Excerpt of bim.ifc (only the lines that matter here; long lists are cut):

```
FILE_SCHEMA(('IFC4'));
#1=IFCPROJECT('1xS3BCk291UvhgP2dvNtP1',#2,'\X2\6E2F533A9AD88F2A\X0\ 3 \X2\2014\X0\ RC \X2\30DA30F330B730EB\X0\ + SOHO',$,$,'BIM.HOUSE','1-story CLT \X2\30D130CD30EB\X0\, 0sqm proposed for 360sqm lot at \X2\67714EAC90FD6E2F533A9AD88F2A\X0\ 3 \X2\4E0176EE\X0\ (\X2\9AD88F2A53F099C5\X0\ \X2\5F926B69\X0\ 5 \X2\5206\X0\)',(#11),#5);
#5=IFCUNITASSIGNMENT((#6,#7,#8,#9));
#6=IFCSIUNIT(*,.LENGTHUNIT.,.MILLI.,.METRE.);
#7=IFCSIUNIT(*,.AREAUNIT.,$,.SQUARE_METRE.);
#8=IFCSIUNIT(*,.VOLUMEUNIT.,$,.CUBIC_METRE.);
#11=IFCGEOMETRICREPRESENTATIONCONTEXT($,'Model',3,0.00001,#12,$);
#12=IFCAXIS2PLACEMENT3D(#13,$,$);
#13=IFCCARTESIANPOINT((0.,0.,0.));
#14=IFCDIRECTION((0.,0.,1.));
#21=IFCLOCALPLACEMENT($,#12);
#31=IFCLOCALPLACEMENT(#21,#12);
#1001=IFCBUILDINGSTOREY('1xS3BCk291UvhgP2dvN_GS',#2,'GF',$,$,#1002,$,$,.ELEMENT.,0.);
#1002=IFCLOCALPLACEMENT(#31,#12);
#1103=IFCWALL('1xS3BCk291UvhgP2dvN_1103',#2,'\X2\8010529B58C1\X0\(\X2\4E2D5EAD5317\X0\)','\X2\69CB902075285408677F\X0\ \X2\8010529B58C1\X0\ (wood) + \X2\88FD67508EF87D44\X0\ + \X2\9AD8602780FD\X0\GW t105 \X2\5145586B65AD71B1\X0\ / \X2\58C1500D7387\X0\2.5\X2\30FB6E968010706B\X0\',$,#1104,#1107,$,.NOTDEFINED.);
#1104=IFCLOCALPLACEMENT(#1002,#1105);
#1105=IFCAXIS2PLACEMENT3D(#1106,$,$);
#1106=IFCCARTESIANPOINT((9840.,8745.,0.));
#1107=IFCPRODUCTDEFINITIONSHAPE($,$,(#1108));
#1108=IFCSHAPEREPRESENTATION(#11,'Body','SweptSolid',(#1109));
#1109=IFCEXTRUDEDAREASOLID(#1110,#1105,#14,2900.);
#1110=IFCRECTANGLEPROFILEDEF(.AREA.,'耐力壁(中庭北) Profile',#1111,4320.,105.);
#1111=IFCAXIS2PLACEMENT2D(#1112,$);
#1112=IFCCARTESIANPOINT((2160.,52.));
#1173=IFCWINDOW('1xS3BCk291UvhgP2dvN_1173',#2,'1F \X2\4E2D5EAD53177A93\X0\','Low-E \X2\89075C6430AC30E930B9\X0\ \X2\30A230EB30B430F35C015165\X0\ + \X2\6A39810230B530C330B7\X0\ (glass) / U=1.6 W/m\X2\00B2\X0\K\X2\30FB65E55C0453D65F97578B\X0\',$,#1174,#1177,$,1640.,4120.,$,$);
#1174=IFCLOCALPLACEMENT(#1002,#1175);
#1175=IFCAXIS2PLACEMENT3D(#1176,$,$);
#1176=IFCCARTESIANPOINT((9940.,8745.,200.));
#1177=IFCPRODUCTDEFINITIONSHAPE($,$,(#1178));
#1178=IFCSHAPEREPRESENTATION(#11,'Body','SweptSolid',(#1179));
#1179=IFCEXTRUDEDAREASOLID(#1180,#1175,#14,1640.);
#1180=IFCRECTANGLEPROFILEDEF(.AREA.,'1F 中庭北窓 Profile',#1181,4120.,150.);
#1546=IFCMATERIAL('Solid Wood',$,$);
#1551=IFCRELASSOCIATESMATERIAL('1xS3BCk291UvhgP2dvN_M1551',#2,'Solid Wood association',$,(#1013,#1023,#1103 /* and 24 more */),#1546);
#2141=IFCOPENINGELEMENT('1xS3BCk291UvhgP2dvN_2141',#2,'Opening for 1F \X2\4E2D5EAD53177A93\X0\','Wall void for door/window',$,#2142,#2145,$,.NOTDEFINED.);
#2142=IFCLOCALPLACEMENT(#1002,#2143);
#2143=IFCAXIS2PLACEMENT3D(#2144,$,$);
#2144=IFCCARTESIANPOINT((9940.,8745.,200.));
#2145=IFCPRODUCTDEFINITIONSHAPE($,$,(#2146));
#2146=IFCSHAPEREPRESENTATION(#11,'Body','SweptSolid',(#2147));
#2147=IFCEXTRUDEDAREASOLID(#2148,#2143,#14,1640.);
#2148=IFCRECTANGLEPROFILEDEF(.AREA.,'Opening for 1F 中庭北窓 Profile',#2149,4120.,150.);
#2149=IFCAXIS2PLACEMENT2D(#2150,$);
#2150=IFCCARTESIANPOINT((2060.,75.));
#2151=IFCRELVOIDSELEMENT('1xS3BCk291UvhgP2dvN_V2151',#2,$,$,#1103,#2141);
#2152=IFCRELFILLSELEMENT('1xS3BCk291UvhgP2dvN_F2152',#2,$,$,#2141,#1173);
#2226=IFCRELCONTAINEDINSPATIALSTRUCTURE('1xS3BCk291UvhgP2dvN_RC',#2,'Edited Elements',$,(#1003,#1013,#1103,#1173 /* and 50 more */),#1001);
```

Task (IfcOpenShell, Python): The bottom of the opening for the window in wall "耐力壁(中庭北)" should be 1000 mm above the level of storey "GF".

```python
import numpy as np
import ifcopenshell
import ifcopenshell.api.geometry
import ifcopenshell.geom
import ifcopenshell.util.element
import ifcopenshell.util.placement
import ifcopenshell.util.shape
import ifcopenshell.util.unit

model = ifcopenshell.open("bim.ifc")
unit_scale = ifcopenshell.util.unit.calculate_unit_scale(model)

window = model.by_id(1173)
opening = window.FillsVoids[0].RelatingOpeningElement
storey = ifcopenshell.util.element.get_container(window, ifc_class="IfcBuildingStorey")
level = ifcopenshell.util.placement.get_local_placement(storey.ObjectPlacement)[2, 3]

# The opening's origin need not be at the sill, so measure its lowest point.
shape = ifcopenshell.geom.create_shape(ifcopenshell.geom.settings(), opening)
bottom = ifcopenshell.util.shape.get_shape_bottom_elevation(shape, shape.geometry) / unit_scale
dz = level + 1000.0 - bottom

shift = np.array([0.0, 0.0, dz])
# The window is not placed relative to its opening, so move both.
for product in (opening, window):
    matrix = ifcopenshell.util.placement.get_local_placement(product.ObjectPlacement)
    matrix[:3, 3] += shift
    ifcopenshell.api.geometry.edit_object_placement(model, product=product, matrix=matrix, is_si=False)

print(f"moved by {dz * unit_scale:+.3f} m")

model.write("bim_v2.ifc")
```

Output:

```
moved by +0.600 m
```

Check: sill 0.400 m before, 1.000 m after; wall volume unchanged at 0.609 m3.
